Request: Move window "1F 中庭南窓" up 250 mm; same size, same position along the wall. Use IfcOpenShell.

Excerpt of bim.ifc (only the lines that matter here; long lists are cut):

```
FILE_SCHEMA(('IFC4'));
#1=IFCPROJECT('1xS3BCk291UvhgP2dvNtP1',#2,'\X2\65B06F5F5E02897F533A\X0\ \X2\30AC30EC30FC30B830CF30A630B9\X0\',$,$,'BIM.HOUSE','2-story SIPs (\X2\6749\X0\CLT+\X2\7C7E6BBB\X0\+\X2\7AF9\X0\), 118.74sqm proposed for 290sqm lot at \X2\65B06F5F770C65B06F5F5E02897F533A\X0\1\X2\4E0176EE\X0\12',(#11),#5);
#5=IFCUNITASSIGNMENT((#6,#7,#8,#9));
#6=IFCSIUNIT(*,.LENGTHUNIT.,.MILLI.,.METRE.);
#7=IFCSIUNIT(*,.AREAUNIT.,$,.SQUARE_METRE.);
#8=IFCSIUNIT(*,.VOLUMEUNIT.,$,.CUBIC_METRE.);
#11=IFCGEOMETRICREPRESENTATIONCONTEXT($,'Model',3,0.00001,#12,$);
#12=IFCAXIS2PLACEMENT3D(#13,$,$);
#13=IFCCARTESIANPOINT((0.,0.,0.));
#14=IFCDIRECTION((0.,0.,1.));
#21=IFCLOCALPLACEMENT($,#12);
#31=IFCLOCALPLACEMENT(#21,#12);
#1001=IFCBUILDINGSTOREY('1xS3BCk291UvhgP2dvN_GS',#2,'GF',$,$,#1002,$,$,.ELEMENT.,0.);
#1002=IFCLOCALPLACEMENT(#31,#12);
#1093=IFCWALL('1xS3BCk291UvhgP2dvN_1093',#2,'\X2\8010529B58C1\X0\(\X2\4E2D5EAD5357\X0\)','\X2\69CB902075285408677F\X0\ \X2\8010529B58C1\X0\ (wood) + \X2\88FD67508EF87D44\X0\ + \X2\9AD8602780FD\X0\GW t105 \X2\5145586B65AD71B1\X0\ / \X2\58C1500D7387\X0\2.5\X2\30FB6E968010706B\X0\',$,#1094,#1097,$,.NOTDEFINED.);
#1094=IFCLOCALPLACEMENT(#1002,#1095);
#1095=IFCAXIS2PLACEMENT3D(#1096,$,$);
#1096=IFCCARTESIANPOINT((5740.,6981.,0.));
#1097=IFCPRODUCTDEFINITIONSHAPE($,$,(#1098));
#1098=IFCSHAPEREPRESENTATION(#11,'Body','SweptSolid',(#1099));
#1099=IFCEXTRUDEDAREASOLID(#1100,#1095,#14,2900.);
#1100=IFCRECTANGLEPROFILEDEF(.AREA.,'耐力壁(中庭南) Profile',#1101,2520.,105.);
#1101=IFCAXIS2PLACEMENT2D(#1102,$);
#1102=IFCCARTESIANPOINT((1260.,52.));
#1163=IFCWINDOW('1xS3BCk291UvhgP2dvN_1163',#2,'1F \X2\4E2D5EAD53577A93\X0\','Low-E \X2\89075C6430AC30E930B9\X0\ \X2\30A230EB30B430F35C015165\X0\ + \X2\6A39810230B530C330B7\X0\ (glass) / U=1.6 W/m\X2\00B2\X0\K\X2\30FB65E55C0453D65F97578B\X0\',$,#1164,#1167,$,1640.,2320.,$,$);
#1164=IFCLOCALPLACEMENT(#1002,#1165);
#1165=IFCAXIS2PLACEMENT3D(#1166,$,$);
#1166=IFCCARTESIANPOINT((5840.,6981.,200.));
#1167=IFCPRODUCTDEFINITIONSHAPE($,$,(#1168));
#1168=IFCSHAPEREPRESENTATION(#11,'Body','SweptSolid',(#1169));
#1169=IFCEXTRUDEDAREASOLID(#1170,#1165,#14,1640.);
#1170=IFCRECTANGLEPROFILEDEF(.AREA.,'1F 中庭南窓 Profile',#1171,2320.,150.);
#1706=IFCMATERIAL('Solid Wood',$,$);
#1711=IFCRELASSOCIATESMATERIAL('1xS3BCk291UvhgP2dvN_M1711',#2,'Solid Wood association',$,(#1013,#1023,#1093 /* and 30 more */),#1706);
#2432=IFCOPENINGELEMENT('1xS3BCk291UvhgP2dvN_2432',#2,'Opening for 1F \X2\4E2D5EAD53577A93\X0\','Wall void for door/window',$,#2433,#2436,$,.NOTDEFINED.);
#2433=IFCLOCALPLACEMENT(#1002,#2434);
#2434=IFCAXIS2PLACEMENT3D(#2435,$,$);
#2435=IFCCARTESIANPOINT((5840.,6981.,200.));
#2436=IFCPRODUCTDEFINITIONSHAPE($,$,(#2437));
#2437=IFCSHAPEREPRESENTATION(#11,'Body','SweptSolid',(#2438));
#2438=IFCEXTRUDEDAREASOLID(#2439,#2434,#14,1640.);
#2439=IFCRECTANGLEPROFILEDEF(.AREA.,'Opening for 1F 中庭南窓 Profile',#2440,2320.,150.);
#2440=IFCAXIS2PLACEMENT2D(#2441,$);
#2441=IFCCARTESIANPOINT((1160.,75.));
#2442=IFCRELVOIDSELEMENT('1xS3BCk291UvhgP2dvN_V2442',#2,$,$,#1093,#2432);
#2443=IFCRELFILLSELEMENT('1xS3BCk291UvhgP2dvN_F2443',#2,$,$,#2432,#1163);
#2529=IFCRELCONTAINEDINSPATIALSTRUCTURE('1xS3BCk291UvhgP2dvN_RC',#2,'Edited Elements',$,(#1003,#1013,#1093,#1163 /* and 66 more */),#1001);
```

```python
import numpy as np
import ifcopenshell
import ifcopenshell.api.geometry
import ifcopenshell.util.placement
import ifcopenshell.util.unit

model = ifcopenshell.open("bim.ifc")
unit_scale = ifcopenshell.util.unit.calculate_unit_scale(model)

window = model.by_id(1163)
opening = window.FillsVoids[0].RelatingOpeningElement
dz = 0.25 / unit_scale

shift = np.array([0.0, 0.0, dz])
# The window is not placed relative to its opening, so move both.
for product in (opening, window):
    matrix = ifcopenshell.util.placement.get_local_placement(product.ObjectPlacement)
    matrix[:3, 3] += shift
    ifcopenshell.api.geometry.edit_object_placement(model, product=product, matrix=matrix, is_si=False)

print(f"moved by {dz * unit_scale:+.3f} m")

model.write("bim_v2.ifc")
```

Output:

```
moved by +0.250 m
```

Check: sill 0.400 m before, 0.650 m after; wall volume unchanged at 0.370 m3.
